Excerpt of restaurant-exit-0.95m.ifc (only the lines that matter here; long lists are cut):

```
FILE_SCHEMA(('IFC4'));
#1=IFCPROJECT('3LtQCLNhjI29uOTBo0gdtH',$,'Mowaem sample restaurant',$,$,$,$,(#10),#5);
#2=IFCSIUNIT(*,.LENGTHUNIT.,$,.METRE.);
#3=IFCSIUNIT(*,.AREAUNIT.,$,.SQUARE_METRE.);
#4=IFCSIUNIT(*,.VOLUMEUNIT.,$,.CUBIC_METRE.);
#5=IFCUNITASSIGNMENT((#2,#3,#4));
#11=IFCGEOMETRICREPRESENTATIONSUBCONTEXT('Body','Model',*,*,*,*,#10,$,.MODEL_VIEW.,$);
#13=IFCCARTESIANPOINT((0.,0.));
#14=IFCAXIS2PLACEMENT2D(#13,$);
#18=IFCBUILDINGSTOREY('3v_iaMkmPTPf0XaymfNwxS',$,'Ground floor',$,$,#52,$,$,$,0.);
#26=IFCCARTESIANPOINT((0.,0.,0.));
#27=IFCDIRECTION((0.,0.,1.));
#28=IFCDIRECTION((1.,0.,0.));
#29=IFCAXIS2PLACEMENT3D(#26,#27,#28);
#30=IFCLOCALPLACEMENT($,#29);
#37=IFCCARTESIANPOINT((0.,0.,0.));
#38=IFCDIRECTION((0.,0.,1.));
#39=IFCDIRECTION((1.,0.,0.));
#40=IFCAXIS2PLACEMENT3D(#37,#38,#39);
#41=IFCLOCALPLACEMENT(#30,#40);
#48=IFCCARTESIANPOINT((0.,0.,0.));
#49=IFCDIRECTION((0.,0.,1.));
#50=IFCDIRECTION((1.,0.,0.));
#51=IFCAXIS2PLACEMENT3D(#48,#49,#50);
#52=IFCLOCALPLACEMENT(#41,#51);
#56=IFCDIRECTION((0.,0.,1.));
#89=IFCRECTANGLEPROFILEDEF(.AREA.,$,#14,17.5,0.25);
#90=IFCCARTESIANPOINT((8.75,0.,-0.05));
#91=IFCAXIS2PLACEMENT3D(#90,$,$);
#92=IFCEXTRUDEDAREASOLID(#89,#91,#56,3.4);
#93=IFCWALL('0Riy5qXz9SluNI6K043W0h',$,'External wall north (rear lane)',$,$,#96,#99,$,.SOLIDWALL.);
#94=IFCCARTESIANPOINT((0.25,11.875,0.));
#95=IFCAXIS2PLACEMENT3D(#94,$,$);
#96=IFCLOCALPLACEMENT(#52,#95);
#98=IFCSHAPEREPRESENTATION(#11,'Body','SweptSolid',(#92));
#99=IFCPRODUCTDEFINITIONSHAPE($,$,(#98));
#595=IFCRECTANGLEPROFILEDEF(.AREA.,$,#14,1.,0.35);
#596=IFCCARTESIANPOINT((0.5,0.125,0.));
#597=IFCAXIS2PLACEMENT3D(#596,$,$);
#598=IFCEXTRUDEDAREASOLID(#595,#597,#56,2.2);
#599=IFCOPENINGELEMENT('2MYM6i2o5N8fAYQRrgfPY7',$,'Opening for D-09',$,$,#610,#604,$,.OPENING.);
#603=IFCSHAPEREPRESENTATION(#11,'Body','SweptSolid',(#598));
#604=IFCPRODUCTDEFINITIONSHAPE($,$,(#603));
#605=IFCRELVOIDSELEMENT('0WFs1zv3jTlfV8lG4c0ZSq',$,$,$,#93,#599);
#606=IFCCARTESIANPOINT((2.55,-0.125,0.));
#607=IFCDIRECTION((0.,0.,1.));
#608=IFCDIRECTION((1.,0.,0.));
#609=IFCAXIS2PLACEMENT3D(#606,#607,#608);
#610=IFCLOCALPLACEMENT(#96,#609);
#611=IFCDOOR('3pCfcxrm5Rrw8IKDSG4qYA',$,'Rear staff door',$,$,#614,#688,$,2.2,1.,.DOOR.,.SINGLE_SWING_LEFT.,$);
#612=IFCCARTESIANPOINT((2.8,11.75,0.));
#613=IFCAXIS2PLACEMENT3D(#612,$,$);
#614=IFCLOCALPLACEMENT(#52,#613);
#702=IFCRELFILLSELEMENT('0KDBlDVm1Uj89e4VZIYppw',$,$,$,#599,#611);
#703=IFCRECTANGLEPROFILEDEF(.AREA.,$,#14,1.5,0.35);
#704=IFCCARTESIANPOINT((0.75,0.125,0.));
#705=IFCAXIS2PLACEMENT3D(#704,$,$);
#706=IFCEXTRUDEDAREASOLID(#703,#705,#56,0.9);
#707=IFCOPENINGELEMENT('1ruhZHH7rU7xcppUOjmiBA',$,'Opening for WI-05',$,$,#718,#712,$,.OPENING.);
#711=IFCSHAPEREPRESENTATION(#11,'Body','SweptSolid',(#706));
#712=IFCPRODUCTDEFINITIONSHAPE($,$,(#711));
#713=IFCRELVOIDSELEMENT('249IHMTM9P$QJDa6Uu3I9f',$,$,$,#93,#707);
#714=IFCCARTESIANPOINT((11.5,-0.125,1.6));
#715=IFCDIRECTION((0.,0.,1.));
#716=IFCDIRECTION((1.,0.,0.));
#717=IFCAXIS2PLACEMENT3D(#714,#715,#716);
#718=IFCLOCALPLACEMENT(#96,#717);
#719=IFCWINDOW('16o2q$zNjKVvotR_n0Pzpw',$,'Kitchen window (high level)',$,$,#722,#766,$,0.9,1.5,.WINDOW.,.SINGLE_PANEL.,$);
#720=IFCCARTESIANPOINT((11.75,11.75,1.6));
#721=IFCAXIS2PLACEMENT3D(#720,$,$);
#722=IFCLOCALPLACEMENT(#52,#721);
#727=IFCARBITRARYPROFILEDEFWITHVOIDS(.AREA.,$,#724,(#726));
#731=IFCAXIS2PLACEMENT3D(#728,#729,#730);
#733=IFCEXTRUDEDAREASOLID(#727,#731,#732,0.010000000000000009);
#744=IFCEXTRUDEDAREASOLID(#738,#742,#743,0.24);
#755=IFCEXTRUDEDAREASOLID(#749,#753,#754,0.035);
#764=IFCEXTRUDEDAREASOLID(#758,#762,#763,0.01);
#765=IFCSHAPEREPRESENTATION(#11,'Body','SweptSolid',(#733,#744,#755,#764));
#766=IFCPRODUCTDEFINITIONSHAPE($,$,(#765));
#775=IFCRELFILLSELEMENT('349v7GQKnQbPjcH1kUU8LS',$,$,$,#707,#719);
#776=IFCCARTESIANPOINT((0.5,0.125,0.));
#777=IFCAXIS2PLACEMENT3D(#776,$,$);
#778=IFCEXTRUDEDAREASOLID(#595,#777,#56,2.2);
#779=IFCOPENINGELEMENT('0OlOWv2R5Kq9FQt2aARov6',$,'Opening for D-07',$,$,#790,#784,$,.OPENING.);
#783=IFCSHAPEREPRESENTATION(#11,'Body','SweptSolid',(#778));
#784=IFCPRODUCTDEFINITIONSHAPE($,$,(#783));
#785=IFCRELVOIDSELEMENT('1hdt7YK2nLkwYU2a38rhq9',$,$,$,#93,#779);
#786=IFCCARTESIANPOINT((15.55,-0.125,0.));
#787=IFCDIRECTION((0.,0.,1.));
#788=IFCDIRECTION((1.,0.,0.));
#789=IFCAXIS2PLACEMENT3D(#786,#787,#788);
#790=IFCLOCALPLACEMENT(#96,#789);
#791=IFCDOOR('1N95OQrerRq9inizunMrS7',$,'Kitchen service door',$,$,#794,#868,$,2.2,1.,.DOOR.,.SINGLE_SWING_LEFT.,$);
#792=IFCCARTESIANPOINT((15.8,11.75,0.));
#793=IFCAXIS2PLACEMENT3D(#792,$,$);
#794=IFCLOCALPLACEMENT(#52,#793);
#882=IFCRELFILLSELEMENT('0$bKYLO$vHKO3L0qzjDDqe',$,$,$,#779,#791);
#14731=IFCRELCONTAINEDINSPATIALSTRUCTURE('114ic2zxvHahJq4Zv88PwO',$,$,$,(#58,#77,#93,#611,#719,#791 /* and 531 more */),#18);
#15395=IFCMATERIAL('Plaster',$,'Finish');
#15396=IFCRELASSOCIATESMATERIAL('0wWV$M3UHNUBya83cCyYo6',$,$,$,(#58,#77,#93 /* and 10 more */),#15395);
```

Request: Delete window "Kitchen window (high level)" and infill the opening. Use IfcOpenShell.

```python
import ifcopenshell
import ifcopenshell.api.feature
import ifcopenshell.api.root
import ifcopenshell.geom
import ifcopenshell.util.shape

model = ifcopenshell.open("restaurant-exit-0.95m.ifc")
settings = ifcopenshell.geom.settings()


def volume(element):
    """Net volume in cubic metres, openings subtracted."""
    shape = ifcopenshell.geom.create_shape(settings, element)
    return ifcopenshell.util.shape.get_volume(shape.geometry)


window = model.by_guid("16o2q$zNjKVvotR_n0Pzpw")
opening = window.FillsVoids[0].RelatingOpeningElement
wall = opening.VoidsElements[0].RelatingBuildingElement
before = volume(wall)

ifcopenshell.api.root.remove_product(model, product=window)
ifcopenshell.api.feature.remove_feature(model, feature=opening)

after = volume(wall)

print(f"wall volume {before:.3f} -> {after:.3f} m3")

model.write("restaurant-exit-0.95m_v2.ifc")
```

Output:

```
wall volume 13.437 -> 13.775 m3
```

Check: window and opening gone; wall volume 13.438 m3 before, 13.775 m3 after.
